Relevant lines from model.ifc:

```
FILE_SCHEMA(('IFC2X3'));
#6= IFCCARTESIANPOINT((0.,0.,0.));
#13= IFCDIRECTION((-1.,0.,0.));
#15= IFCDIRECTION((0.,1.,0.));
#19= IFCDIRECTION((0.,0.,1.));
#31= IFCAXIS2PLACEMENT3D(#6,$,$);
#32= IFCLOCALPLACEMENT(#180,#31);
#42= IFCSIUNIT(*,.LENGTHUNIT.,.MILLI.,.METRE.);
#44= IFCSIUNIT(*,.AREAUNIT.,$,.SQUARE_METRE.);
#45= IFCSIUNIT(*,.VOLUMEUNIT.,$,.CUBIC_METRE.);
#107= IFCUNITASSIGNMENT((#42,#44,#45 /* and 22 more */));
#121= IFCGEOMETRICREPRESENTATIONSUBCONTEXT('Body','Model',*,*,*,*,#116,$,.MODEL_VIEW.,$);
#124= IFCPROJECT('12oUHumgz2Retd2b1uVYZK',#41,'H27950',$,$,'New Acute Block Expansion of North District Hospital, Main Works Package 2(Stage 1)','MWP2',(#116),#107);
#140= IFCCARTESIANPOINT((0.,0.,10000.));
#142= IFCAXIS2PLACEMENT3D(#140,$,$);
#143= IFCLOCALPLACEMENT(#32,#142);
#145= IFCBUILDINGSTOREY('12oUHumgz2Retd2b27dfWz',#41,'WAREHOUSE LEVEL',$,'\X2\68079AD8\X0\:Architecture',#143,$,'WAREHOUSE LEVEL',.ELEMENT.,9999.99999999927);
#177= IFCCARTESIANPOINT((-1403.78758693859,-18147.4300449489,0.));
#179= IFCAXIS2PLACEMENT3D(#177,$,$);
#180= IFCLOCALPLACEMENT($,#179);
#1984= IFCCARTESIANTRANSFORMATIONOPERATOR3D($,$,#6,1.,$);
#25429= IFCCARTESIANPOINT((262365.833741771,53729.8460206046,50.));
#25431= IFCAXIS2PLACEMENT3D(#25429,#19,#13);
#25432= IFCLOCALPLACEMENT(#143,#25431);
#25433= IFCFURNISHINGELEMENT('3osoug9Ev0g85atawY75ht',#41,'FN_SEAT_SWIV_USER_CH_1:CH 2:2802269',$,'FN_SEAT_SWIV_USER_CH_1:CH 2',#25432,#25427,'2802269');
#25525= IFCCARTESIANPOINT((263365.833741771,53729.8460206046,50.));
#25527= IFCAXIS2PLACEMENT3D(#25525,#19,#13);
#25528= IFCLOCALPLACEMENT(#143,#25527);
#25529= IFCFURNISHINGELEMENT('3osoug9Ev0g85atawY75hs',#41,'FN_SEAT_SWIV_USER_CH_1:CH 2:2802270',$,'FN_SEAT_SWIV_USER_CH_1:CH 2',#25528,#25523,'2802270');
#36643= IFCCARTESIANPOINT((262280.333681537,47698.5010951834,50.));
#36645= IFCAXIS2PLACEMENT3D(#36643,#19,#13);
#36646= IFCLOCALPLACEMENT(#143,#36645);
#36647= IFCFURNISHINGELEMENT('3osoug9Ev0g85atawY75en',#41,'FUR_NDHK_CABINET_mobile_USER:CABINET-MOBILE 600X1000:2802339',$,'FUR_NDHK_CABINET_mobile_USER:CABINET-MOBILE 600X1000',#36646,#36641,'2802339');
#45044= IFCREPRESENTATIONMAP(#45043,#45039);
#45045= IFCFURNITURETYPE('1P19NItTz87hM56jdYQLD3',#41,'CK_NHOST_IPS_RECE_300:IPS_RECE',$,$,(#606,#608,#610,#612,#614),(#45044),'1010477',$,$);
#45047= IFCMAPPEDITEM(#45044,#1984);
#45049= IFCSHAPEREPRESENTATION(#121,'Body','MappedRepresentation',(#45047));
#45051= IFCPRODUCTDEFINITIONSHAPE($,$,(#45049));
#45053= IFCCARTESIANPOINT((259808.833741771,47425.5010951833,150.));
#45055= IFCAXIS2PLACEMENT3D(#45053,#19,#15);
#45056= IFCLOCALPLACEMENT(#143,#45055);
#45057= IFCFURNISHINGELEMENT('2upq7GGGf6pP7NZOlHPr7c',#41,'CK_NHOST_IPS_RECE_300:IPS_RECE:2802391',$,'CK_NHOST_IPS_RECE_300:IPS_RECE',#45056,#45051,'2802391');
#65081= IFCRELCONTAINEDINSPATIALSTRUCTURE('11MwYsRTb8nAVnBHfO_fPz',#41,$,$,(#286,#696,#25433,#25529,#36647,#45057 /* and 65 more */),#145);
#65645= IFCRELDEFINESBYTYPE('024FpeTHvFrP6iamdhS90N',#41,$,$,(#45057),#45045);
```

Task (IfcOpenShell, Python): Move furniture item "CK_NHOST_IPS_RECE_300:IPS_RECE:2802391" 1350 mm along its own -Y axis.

```python
import ifcopenshell
import ifcopenshell.api.geometry
import ifcopenshell.util.placement

model = ifcopenshell.open("model.ifc")

item = model.by_guid("2upq7GGGf6pP7NZOlHPr7c")
matrix = ifcopenshell.util.placement.get_local_placement(item.ObjectPlacement)
matrix[:3, 3] -= matrix[:3, 1] * 1350.0
ifcopenshell.api.geometry.edit_object_placement(model, product=item, matrix=matrix, is_si=False)

print(ifcopenshell.util.placement.get_local_placement(item.ObjectPlacement).round(3) + 0.0)

model.write("model-out.ifc")
```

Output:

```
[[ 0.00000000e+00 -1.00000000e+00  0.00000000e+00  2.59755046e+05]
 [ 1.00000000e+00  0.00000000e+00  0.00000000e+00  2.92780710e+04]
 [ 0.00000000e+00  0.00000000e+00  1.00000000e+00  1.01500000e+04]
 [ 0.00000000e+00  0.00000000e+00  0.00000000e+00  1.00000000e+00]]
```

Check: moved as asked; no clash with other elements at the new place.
